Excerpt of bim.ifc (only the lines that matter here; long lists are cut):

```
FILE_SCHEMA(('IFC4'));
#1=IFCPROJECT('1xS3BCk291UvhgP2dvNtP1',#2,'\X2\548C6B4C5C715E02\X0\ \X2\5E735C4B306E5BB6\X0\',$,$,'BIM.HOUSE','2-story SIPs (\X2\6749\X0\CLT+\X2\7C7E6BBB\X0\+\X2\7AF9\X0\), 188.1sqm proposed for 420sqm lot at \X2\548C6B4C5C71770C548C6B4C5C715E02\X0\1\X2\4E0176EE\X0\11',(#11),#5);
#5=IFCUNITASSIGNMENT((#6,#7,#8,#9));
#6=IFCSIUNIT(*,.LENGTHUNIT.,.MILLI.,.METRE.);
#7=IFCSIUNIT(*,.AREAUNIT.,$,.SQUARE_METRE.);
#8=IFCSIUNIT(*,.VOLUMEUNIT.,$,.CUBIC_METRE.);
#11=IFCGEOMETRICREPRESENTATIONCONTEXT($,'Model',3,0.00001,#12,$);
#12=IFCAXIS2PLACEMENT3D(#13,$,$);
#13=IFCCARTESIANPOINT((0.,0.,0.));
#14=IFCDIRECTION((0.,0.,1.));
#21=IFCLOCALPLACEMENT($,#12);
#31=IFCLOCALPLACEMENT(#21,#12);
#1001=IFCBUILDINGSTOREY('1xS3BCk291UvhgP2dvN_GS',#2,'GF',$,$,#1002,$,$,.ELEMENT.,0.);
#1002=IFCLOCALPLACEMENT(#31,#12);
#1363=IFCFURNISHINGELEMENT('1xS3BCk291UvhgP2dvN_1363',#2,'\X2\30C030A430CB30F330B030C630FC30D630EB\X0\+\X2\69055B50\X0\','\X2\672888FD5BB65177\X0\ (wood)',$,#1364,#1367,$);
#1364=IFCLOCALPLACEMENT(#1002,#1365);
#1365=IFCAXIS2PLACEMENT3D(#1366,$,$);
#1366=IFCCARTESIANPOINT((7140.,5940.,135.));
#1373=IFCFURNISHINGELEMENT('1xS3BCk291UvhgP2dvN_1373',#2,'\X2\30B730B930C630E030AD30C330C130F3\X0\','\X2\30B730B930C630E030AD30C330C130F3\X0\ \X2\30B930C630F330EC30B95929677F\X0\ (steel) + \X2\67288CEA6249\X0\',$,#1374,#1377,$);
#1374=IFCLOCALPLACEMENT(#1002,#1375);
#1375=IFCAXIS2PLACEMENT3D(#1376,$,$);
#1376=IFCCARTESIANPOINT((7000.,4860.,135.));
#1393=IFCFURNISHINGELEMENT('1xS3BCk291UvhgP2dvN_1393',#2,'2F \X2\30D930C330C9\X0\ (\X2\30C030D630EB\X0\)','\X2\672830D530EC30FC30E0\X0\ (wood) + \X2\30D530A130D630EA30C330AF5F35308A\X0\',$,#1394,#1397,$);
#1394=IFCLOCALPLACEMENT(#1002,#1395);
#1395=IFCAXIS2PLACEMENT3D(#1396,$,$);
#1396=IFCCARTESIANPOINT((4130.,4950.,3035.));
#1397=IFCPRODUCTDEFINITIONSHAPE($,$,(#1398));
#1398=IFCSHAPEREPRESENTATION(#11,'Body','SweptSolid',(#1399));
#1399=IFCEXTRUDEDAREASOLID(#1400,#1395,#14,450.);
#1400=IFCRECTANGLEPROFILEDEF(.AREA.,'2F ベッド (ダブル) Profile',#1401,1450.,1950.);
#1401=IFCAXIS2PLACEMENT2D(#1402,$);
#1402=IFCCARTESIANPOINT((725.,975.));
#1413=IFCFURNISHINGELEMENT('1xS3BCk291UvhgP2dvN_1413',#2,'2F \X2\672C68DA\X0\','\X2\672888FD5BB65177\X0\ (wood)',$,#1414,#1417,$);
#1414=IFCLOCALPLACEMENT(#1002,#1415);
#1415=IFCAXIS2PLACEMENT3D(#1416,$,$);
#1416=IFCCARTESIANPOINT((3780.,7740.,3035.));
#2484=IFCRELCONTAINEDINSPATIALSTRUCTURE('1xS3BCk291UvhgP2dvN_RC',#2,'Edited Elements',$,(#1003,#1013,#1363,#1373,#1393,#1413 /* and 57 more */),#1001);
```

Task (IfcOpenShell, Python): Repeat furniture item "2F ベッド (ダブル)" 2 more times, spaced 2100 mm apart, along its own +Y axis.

```python
import ifcopenshell
import ifcopenshell.api.geometry
import ifcopenshell.api.root
import ifcopenshell.util.element
import ifcopenshell.util.placement
import ifcopenshell.util.unit

model = ifcopenshell.open("bim.ifc")
unit_scale = ifcopenshell.util.unit.calculate_unit_scale(model)


def reuse_history(source, copy):
    """copy_class also copies each property set's owner history, people and application; keep the originals."""
    for rel in copy.IsDefinedBy:
        if rel.is_a("IfcRelDefinesByProperties") and (history := rel.RelatingPropertyDefinition.OwnerHistory):
            rel.RelatingPropertyDefinition.OwnerHistory = source.OwnerHistory
            ifcopenshell.util.element.remove_deep2(model, history)


source = model.by_guid("1xS3BCk291UvhgP2dvN_1393")
base = ifcopenshell.util.placement.get_local_placement(source.ObjectPlacement)
step = base[:3, 1] * 2.1 / unit_scale

for i in range(1, 3):
    copy = ifcopenshell.api.root.copy_class(model, product=source)
    copy.Representation = ifcopenshell.util.element.copy_deep(
        model, source.Representation, exclude=["IfcGeometricRepresentationContext", "IfcRepresentationMap"]
    )
    reuse_history(source, copy)
    matrix = base.copy()
    matrix[:3, 3] += i * step
    print("added at", matrix[:3, 3].round(3) + 0.0)
    ifcopenshell.api.geometry.edit_object_placement(model, product=copy, matrix=matrix, is_si=False)

model.write("bim-out.ifc")
```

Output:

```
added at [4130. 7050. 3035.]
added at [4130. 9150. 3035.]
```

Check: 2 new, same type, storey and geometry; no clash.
